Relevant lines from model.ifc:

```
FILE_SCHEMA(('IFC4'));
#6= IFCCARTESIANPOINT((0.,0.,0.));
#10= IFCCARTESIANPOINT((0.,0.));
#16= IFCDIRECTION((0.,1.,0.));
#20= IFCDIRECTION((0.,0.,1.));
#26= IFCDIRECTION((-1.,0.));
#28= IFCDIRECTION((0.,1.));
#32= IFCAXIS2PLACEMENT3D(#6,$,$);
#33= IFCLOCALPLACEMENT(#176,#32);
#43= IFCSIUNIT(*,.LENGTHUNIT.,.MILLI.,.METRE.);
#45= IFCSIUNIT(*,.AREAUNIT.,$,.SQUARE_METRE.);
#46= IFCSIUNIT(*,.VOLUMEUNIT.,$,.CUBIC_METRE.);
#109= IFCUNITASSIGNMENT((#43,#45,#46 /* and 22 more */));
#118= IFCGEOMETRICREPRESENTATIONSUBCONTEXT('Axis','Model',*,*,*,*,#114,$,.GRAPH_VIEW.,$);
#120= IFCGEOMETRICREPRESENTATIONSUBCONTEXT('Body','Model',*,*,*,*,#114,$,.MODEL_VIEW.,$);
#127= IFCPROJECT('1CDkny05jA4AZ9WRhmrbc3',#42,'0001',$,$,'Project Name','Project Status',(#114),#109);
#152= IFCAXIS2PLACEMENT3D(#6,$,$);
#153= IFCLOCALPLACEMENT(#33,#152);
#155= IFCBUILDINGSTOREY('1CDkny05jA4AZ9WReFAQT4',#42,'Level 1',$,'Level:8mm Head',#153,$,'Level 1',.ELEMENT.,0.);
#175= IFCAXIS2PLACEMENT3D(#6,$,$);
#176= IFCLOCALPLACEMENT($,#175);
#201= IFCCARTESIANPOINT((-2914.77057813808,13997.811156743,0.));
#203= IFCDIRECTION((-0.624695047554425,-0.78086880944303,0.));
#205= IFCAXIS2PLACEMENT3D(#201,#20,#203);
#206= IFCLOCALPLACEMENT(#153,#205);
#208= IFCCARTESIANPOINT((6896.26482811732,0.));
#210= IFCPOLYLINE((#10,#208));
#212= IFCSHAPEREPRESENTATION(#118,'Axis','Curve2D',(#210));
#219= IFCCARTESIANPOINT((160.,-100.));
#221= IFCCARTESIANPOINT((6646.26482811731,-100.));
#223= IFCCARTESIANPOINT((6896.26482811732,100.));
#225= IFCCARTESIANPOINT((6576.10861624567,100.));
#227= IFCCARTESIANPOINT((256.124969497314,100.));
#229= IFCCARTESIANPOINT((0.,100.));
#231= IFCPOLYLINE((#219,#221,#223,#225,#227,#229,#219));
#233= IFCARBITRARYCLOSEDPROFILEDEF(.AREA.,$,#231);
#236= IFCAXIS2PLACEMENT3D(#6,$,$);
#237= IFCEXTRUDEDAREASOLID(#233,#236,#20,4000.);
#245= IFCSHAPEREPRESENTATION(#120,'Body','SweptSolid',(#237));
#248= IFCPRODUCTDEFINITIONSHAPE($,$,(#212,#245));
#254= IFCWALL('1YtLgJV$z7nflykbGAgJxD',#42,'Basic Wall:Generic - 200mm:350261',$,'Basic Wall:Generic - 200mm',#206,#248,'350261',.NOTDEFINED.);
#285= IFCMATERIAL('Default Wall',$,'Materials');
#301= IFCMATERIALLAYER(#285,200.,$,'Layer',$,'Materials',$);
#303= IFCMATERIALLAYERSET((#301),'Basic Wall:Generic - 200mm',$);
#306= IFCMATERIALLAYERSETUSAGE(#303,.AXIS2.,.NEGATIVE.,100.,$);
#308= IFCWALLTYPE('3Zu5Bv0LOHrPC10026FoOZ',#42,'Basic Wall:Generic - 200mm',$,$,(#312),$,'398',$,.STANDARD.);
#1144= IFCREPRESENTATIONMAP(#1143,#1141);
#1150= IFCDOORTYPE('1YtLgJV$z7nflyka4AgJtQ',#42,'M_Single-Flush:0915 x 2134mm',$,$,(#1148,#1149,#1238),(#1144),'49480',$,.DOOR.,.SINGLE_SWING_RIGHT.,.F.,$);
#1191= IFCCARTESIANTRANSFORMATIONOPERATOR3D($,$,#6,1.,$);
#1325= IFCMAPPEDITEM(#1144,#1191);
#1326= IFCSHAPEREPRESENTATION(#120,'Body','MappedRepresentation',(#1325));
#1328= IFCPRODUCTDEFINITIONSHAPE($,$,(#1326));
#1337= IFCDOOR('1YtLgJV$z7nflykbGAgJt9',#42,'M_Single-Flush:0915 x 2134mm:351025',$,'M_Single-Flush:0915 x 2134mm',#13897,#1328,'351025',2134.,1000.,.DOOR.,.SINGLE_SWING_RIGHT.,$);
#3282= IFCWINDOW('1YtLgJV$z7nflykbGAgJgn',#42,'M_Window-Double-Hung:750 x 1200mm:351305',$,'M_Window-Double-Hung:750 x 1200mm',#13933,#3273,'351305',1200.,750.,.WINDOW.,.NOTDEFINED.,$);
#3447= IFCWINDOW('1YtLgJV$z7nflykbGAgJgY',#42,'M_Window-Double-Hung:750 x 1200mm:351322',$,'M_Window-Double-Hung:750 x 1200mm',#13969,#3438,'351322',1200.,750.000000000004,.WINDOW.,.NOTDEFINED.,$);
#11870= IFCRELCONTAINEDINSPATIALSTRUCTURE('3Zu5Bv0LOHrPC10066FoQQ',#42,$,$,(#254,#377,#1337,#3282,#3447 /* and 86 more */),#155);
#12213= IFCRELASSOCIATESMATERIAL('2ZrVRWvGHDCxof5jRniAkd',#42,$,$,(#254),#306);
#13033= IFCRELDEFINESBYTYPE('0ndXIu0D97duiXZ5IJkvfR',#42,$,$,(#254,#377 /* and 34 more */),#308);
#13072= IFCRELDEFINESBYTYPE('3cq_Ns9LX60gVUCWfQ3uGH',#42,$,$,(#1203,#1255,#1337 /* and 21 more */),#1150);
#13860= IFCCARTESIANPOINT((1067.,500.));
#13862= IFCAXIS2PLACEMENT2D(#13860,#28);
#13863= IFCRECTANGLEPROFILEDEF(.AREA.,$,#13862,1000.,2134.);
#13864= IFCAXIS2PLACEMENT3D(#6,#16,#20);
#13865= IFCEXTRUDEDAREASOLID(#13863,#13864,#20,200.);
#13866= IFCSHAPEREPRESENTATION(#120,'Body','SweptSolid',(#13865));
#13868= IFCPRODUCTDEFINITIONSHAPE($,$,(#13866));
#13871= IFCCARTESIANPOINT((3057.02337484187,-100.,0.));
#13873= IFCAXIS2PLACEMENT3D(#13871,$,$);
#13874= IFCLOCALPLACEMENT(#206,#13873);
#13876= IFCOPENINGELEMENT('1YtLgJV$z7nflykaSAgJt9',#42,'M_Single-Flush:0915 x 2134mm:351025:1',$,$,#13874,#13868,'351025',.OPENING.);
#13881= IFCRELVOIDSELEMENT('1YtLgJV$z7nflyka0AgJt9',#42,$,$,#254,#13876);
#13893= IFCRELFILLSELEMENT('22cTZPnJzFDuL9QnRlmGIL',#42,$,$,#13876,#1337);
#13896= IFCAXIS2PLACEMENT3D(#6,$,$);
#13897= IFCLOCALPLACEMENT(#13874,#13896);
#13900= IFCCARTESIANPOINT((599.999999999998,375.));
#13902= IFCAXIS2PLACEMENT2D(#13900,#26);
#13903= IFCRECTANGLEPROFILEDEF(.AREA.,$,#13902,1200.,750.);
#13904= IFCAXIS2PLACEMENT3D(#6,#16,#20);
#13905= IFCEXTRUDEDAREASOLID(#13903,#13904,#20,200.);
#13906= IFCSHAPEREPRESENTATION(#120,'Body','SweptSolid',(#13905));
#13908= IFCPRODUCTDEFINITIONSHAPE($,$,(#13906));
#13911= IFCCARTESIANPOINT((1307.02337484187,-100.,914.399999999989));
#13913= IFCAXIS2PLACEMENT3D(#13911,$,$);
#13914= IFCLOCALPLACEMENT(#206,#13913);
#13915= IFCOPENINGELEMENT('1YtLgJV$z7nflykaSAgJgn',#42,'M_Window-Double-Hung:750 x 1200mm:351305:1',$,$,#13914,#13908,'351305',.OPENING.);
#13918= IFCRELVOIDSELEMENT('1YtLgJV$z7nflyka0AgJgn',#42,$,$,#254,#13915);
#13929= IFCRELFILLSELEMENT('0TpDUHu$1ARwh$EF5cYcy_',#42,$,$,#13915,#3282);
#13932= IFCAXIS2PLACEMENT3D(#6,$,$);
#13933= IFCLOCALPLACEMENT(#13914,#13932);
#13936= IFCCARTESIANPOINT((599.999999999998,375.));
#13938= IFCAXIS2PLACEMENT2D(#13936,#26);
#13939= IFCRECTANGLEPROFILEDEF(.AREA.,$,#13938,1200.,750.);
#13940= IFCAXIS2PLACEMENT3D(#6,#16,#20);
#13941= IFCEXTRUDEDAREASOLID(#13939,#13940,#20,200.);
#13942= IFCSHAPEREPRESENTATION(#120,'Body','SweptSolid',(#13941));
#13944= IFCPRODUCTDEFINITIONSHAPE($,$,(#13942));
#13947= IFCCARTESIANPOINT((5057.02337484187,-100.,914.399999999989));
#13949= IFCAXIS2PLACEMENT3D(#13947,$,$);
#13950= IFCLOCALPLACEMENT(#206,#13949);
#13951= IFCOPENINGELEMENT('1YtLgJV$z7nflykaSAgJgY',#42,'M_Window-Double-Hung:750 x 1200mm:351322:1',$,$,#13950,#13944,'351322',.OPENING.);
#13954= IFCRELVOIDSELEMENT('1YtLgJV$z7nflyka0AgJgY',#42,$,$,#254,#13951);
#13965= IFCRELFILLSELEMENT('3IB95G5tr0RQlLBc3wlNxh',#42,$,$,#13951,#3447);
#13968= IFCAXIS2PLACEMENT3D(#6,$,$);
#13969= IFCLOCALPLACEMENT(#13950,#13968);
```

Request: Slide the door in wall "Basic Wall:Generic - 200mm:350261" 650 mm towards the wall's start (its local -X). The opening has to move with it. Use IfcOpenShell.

```python
import ifcopenshell
import ifcopenshell.api.geometry
import ifcopenshell.util.placement
import ifcopenshell.util.unit

model = ifcopenshell.open("model.ifc")
unit_scale = ifcopenshell.util.unit.calculate_unit_scale(model)

door = model.by_guid("1YtLgJV$z7nflykbGAgJt9")
opening = door.FillsVoids[0].RelatingOpeningElement
wall = opening.VoidsElements[0].RelatingBuildingElement

wall_matrix = ifcopenshell.util.placement.get_local_placement(wall.ObjectPlacement)
shift = wall_matrix[:3, 0] * -0.65 / unit_scale
before = ifcopenshell.util.placement.get_local_placement(door.ObjectPlacement)[:3, 3].copy()

# The door is placed relative to its opening, so it follows when the opening moves.
matrix = ifcopenshell.util.placement.get_local_placement(opening.ObjectPlacement)
matrix[:3, 3] += shift
ifcopenshell.api.geometry.edit_object_placement(
    model, product=opening, matrix=matrix, is_si=False, should_transform_children=True
)

after = ifcopenshell.util.placement.get_local_placement(door.ObjectPlacement)[:3, 3]
print("door moved by", (after - before).round(3) + 0.0)

model.write("model_edited.ifc")
```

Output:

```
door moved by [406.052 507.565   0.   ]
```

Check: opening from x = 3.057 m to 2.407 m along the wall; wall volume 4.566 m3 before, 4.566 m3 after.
